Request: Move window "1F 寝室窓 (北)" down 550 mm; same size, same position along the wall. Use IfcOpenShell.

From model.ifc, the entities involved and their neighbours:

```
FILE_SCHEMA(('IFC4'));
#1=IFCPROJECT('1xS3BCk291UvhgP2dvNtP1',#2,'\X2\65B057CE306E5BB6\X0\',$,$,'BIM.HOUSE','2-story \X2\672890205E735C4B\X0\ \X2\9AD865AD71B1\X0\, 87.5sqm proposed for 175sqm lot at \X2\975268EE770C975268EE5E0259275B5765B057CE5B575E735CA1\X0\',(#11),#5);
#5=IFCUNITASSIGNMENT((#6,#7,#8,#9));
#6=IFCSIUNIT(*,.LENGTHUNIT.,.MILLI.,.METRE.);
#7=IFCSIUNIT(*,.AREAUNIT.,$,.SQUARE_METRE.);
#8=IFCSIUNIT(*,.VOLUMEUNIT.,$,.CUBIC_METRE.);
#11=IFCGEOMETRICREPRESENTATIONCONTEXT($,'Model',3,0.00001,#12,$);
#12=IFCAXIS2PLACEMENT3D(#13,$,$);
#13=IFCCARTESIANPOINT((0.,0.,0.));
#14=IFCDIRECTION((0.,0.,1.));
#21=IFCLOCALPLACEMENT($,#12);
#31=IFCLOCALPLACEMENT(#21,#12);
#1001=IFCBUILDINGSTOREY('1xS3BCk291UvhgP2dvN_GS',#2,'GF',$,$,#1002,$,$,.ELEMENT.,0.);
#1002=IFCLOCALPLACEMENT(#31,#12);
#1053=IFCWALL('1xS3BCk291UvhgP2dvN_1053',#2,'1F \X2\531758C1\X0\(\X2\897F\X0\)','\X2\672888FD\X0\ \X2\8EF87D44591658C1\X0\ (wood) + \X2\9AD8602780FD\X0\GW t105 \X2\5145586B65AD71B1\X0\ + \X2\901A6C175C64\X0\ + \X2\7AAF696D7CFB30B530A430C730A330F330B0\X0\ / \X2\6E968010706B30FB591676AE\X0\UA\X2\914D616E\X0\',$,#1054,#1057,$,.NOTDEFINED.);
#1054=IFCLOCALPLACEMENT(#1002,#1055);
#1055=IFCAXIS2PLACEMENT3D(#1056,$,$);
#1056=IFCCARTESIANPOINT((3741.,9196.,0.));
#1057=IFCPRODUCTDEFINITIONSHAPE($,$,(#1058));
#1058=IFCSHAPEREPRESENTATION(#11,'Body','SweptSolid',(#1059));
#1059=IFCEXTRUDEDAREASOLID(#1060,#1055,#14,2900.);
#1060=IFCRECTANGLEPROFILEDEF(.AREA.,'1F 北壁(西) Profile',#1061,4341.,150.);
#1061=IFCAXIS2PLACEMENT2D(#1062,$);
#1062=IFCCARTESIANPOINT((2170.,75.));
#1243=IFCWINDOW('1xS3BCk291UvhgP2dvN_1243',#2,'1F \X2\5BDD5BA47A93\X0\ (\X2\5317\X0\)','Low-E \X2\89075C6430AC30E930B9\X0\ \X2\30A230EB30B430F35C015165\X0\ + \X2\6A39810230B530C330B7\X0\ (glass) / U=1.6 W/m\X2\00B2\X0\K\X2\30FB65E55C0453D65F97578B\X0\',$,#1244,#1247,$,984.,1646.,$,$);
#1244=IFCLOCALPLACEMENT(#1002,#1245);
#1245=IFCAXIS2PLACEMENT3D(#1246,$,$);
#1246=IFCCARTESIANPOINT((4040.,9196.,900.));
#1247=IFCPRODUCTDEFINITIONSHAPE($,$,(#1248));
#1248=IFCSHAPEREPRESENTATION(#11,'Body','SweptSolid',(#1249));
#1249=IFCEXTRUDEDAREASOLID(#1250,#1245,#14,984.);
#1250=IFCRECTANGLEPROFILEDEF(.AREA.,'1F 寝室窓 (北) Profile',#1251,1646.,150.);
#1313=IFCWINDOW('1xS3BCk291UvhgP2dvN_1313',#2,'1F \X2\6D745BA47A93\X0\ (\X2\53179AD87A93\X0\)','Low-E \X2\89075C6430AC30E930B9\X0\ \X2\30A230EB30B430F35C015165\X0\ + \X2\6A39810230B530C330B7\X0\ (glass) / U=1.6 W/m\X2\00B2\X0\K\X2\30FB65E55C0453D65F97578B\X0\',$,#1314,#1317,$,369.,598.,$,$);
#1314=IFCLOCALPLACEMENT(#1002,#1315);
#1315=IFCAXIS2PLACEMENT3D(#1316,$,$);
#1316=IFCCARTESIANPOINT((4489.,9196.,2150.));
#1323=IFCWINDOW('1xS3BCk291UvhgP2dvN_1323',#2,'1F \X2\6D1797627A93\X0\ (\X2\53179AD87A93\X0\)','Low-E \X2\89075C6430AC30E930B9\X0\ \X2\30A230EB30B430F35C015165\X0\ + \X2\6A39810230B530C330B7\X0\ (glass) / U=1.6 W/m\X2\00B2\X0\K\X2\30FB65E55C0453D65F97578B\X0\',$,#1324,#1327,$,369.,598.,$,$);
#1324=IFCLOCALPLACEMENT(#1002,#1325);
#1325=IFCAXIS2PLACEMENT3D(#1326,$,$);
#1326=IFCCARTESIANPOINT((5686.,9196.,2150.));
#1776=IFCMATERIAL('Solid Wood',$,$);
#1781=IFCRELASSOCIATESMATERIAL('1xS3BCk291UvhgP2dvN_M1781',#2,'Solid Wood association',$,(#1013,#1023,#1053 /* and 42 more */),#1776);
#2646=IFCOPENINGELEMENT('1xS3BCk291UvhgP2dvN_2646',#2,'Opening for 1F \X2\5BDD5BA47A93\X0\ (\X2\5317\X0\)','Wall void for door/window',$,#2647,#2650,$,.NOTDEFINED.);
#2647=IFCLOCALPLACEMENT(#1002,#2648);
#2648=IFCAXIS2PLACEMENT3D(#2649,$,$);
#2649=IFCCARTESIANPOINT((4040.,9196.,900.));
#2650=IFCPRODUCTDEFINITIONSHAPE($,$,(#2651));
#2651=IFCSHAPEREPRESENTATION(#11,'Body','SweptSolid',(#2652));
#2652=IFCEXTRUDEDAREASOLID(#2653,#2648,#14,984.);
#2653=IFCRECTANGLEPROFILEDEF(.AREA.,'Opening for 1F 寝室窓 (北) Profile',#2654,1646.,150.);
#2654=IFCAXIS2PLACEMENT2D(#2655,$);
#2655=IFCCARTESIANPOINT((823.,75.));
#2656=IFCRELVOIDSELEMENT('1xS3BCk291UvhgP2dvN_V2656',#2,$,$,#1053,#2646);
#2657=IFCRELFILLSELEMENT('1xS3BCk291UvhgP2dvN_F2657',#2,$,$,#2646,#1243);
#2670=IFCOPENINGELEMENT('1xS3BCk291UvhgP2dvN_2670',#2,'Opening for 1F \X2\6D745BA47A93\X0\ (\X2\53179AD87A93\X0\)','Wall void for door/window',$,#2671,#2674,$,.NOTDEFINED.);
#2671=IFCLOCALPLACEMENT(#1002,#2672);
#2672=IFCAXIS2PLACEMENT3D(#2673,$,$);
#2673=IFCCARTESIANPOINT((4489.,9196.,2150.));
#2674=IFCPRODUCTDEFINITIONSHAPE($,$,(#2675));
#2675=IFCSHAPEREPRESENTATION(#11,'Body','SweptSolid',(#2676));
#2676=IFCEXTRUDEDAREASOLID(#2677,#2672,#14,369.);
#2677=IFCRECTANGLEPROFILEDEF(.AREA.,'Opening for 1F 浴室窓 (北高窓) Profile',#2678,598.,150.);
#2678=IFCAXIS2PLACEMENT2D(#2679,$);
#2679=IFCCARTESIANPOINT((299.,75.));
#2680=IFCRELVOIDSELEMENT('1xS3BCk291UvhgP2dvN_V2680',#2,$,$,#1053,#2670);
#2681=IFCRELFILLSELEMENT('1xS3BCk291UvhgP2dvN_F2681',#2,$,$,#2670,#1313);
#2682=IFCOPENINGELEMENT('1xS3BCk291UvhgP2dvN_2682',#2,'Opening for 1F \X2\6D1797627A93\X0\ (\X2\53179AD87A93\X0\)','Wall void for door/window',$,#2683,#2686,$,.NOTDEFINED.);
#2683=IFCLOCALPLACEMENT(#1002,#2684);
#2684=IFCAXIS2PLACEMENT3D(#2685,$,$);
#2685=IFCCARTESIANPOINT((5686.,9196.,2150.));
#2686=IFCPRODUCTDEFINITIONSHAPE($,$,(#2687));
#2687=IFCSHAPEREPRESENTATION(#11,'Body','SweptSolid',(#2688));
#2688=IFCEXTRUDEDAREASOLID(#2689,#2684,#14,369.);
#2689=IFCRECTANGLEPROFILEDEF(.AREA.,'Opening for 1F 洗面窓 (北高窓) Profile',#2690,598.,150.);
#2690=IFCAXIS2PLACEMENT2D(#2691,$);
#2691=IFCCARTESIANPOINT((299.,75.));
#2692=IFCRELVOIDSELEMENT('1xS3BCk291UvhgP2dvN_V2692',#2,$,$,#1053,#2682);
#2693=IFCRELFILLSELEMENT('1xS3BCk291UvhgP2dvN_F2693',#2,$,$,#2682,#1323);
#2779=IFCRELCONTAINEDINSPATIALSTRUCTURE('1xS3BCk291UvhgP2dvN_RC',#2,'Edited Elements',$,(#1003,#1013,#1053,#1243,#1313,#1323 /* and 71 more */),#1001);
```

```python
import numpy as np
import ifcopenshell
import ifcopenshell.api.geometry
import ifcopenshell.util.placement
import ifcopenshell.util.unit

model = ifcopenshell.open("model.ifc")
unit_scale = ifcopenshell.util.unit.calculate_unit_scale(model)

window = model.by_guid("1xS3BCk291UvhgP2dvN_1243")
opening = window.FillsVoids[0].RelatingOpeningElement
dz = -0.55 / unit_scale

shift = np.array([0.0, 0.0, dz])
# The window is not placed relative to its opening, so move both.
for product in (opening, window):
    matrix = ifcopenshell.util.placement.get_local_placement(product.ObjectPlacement)
    matrix[:3, 3] += shift
    ifcopenshell.api.geometry.edit_object_placement(model, product=product, matrix=matrix, is_si=False)

print(f"moved by {dz * unit_scale:+.3f} m")

model.write("model_v2.ifc")
```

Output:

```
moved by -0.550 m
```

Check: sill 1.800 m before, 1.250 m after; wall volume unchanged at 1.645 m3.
